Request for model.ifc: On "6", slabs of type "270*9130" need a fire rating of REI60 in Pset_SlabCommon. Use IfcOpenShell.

First a look at what the model holds.

```python
import ifcopenshell
import ifcopenshell.util.element

model = ifcopenshell.open("model.ifc")
print(model.schema)
storey = next(s for s in model.by_type("IfcBuildingStorey") if s.Name == "6")
slabs = [e for e in ifcopenshell.util.element.get_decomposition(storey) if e.is_a("IfcSlab")]
seen = {}
for e in slabs:
    element_type = ifcopenshell.util.element.get_type(e)
    key = (element_type.Name if element_type != e and element_type else None, ifcopenshell.util.element.get_pset(e, "Pset_SlabCommon", "FireRating"))
    seen[key] = seen.get(key, 0) + 1
for (name, value), count in sorted(seen.items(), key=str):
    print(count, "x", name, "|", value)
```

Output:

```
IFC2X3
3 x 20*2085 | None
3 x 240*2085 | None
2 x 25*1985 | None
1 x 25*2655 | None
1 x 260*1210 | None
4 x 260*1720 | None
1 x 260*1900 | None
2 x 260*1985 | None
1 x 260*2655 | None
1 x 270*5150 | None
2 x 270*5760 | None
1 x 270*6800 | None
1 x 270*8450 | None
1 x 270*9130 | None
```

```python
import ifcopenshell
import ifcopenshell.api.pset
import ifcopenshell.util.element

model = ifcopenshell.open("model.ifc")

storey = next(s for s in model.by_type("IfcBuildingStorey") if s.Name == "6")
slabs = [e for e in ifcopenshell.util.element.get_decomposition(storey) if e.is_a("IfcSlab")]

count = 0
for e in slabs:
    element_type = ifcopenshell.util.element.get_type(e)
    if element_type in (None, e) or element_type.Name != "270*9130":
        continue
    found = ifcopenshell.util.element.get_pset(e, "Pset_SlabCommon", should_inherit=False)
    if found:
        pset = model.by_id(found["id"])
        if len(ifcopenshell.util.element.get_elements_by_pset(pset)) > 1:
            pset = ifcopenshell.api.pset.unshare_pset(model, products=[e], pset=pset)[0]
    else:
        pset = ifcopenshell.api.pset.add_pset(model, product=e, name="Pset_SlabCommon")
    ifcopenshell.api.pset.edit_pset(model, pset=pset, properties={"FireRating": "REI60"})
    count += 1

print(count, "slabs updated")

model.write("model_edited.ifc")
```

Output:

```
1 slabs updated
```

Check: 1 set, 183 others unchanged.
